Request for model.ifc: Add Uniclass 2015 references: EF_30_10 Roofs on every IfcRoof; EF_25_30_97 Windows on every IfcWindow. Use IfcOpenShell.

First a look at what the model holds.

```python
import ifcopenshell

model = ifcopenshell.open("model.ifc")
print(model.schema)
print("classifications:", [c.Name for c in model.by_type("IfcClassification")])
for ifc_class in ("IfcDoor", "IfcRoof", "IfcStair", "IfcWall", "IfcWindow"):
    print(ifc_class, len(model.by_type(ifc_class)))
```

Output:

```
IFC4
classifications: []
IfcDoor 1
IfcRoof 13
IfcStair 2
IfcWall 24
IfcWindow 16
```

```python
import ifcopenshell
import ifcopenshell.api.classification

model = ifcopenshell.open("model.ifc")

system = ifcopenshell.api.classification.add_classification(model, classification="Uniclass 2015")

codes = {
    "IfcRoof": ("EF_30_10", "Roofs"),
    "IfcWindow": ("EF_25_30_97", "Windows"),
}
for ifc_class, (code, name) in codes.items():
    products = model.by_type(ifc_class)
    ifcopenshell.api.classification.add_reference(
        model, products=products, classification=system, identification=code, name=name
    )
    print(code, len(products))

model.write("model-out.ifc")
```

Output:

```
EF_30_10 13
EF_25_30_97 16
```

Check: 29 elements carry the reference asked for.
